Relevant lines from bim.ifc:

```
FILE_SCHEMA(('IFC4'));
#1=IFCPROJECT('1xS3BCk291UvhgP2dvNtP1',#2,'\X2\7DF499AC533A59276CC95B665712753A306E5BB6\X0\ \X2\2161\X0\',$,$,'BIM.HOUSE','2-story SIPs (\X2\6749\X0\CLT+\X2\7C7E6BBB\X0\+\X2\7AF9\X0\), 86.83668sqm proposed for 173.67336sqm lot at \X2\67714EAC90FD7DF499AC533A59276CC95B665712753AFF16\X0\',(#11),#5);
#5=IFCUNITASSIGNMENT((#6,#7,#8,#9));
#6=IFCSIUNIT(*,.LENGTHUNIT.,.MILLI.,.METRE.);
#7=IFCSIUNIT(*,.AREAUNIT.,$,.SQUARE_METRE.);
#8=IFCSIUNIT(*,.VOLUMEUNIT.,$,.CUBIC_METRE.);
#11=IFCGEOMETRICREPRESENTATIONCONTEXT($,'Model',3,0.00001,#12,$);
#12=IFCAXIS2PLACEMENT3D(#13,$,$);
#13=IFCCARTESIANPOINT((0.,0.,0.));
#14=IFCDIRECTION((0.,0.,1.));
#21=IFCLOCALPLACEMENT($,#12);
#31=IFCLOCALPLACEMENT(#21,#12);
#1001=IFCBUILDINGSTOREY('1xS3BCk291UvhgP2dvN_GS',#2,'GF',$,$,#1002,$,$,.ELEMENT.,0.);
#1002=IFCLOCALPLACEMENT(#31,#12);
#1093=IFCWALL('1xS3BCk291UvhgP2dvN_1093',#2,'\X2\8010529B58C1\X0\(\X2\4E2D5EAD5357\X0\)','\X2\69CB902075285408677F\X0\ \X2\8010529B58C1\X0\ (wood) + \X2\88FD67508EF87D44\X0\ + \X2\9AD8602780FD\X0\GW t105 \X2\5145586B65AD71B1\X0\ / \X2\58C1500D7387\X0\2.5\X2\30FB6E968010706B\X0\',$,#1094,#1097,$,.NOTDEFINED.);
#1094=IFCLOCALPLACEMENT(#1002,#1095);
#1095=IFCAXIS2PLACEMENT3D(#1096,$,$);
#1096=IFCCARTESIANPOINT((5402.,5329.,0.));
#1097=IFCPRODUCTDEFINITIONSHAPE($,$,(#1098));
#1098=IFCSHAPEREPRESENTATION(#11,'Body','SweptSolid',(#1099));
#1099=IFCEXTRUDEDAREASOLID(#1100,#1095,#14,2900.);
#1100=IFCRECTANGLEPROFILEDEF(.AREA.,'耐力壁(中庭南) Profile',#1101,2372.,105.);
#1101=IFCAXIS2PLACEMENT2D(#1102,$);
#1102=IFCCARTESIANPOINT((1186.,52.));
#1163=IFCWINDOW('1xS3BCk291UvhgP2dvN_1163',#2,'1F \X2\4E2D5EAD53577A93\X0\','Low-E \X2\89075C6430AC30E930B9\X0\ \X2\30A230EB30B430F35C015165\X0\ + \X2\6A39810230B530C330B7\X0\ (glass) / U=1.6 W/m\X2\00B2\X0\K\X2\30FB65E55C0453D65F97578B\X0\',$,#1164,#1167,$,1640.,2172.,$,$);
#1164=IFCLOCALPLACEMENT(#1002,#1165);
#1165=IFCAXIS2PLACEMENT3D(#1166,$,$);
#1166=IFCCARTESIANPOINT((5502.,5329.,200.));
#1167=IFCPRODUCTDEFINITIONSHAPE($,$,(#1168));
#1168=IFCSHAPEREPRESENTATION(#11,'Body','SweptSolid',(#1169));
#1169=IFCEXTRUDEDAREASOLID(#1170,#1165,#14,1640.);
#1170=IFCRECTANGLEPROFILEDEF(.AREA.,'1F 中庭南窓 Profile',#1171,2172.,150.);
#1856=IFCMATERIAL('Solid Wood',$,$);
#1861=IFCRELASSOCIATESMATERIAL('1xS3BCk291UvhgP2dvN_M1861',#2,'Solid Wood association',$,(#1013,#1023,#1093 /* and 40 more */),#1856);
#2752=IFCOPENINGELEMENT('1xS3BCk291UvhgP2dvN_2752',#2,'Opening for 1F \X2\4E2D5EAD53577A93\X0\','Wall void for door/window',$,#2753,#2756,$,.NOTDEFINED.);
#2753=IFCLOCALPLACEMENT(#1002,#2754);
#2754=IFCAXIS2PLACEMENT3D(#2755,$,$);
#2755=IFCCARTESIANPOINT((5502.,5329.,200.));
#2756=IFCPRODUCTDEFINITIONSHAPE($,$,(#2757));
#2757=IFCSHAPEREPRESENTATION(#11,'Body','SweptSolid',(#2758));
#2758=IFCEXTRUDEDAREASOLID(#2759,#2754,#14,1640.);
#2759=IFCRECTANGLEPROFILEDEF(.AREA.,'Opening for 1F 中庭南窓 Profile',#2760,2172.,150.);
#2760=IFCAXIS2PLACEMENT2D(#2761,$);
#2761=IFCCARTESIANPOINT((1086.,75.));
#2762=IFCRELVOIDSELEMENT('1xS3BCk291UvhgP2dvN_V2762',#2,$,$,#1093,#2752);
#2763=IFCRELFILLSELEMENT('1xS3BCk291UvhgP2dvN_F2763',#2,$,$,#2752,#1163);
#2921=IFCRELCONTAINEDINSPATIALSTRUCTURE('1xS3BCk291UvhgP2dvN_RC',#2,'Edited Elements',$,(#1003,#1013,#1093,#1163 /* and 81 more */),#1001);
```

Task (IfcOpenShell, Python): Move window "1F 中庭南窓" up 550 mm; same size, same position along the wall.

```python
import numpy as np
import ifcopenshell
import ifcopenshell.api.geometry
import ifcopenshell.util.placement
import ifcopenshell.util.unit

model = ifcopenshell.open("bim.ifc")
unit_scale = ifcopenshell.util.unit.calculate_unit_scale(model)

window = model.by_guid("1xS3BCk291UvhgP2dvN_1163")
opening = window.FillsVoids[0].RelatingOpeningElement
dz = 550.0

shift = np.array([0.0, 0.0, dz])
# The window is not placed relative to its opening, so move both.
for product in (opening, window):
    matrix = ifcopenshell.util.placement.get_local_placement(product.ObjectPlacement)
    matrix[:3, 3] += shift
    ifcopenshell.api.geometry.edit_object_placement(model, product=product, matrix=matrix, is_si=False)

print(f"moved by {dz * unit_scale:+.3f} m")

model.write("bim-out.ifc")
```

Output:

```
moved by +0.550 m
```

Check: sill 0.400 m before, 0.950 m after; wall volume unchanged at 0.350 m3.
